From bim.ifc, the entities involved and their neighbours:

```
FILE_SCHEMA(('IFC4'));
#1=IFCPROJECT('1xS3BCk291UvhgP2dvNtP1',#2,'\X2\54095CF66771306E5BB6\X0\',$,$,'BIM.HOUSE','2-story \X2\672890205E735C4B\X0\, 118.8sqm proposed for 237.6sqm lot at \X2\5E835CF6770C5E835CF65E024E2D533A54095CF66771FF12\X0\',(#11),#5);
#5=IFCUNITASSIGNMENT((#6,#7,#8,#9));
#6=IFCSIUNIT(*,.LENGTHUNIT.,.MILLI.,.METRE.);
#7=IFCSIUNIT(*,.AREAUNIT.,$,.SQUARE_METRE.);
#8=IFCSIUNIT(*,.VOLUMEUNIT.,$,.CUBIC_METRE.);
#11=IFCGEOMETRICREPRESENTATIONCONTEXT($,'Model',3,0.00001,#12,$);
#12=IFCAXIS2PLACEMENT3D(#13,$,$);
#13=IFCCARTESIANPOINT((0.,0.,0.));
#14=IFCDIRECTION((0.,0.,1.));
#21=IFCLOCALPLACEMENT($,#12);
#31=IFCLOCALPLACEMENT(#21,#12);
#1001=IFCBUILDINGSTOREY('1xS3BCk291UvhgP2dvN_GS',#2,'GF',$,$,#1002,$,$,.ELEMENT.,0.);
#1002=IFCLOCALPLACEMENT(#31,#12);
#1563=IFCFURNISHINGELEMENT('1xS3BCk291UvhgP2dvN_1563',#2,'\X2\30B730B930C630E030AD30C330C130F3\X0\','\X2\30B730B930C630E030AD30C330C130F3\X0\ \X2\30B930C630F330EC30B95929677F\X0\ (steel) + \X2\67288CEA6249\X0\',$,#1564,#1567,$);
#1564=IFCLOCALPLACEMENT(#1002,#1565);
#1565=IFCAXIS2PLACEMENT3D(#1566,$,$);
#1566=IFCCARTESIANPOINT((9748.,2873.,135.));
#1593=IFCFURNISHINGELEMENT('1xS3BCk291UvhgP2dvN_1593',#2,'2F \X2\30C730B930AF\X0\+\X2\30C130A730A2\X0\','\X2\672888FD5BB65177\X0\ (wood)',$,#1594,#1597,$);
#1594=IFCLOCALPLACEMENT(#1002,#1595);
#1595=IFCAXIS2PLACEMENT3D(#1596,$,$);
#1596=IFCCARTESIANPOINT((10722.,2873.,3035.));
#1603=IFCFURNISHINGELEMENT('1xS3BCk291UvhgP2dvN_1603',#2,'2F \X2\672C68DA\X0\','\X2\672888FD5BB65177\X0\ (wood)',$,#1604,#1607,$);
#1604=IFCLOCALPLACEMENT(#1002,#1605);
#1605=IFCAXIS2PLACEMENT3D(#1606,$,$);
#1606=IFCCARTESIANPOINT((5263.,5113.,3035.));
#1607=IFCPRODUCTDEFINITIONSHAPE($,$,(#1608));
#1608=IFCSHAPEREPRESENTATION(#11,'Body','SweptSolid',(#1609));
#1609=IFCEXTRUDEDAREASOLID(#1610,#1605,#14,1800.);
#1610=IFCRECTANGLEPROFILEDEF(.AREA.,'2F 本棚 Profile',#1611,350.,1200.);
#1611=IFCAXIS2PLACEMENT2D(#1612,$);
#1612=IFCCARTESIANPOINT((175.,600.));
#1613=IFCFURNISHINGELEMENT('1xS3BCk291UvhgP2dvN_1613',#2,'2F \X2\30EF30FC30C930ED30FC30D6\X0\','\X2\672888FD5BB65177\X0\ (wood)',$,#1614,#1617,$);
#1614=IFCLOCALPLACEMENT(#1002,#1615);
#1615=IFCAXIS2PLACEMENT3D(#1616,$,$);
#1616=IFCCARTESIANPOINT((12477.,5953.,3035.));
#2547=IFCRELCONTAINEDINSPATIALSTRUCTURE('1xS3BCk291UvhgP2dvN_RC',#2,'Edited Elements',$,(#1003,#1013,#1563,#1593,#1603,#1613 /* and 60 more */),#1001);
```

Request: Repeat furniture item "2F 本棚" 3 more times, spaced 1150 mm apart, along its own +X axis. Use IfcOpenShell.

```python
import ifcopenshell
import ifcopenshell.api.geometry
import ifcopenshell.api.root
import ifcopenshell.util.element
import ifcopenshell.util.placement

model = ifcopenshell.open("bim.ifc")


def reuse_history(source, copy):
    """copy_class also copies each property set's owner history, people and application; keep the originals."""
    for rel in copy.IsDefinedBy:
        if rel.is_a("IfcRelDefinesByProperties") and (history := rel.RelatingPropertyDefinition.OwnerHistory):
            rel.RelatingPropertyDefinition.OwnerHistory = source.OwnerHistory
            ifcopenshell.util.element.remove_deep2(model, history)


source = model.by_guid("1xS3BCk291UvhgP2dvN_1603")
base = ifcopenshell.util.placement.get_local_placement(source.ObjectPlacement)
step = base[:3, 0] * 1150.0

for i in range(1, 4):
    copy = ifcopenshell.api.root.copy_class(model, product=source)
    copy.Representation = ifcopenshell.util.element.copy_deep(
        model, source.Representation, exclude=["IfcGeometricRepresentationContext", "IfcRepresentationMap"]
    )
    reuse_history(source, copy)
    matrix = base.copy()
    matrix[:3, 3] += i * step
    print("added at", matrix[:3, 3].round(3) + 0.0)
    ifcopenshell.api.geometry.edit_object_placement(model, product=copy, matrix=matrix, is_si=False)

model.write("bim-out.ifc")
```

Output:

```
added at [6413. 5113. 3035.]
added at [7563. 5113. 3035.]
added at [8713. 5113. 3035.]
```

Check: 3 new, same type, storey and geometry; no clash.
